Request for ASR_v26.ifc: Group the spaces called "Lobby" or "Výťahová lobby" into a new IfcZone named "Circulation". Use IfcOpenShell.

First a look at what the model holds.

```python
import ifcopenshell

model = ifcopenshell.open("ASR_v26.ifc")
print(model.schema)
seen = {}
for space in model.by_type("IfcSpace"):
    seen[space.LongName] = seen.get(space.LongName, 0) + 1
for name, count in sorted(seen.items(), key=str):
    print(count, "x", name)
print("zones:", [z.Name for z in model.by_type("IfcZone")][:20])
```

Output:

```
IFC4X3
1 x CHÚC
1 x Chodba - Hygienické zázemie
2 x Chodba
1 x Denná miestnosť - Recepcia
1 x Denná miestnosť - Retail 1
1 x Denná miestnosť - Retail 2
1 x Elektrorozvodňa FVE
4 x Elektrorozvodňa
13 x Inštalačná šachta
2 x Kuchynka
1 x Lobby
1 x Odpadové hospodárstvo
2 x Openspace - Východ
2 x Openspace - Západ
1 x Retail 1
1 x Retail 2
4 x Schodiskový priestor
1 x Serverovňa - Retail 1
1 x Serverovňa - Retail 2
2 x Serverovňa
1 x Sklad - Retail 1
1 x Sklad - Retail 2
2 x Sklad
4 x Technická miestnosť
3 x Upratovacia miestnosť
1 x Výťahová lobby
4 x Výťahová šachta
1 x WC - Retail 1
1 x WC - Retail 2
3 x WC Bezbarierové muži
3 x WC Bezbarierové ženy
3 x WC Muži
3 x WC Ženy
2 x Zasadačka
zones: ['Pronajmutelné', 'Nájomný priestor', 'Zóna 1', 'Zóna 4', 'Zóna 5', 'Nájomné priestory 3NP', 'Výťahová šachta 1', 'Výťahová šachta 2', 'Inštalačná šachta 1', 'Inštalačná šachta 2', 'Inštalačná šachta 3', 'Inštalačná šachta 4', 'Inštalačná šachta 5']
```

```python
import ifcopenshell
import ifcopenshell.api.group
import ifcopenshell.api.root

model = ifcopenshell.open("ASR_v26.ifc")

names = {"Lobby", "Výťahová lobby"}
spaces = [s for s in model.by_type("IfcSpace") if s.LongName in names]

zone = ifcopenshell.api.root.create_entity(model, ifc_class="IfcZone", name="Circulation")
ifcopenshell.api.group.assign_group(model, products=spaces, group=zone)
print(len(spaces), "spaces in", zone.Name)

model.write("ASR_v26-out.ifc")
```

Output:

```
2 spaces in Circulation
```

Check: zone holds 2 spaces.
